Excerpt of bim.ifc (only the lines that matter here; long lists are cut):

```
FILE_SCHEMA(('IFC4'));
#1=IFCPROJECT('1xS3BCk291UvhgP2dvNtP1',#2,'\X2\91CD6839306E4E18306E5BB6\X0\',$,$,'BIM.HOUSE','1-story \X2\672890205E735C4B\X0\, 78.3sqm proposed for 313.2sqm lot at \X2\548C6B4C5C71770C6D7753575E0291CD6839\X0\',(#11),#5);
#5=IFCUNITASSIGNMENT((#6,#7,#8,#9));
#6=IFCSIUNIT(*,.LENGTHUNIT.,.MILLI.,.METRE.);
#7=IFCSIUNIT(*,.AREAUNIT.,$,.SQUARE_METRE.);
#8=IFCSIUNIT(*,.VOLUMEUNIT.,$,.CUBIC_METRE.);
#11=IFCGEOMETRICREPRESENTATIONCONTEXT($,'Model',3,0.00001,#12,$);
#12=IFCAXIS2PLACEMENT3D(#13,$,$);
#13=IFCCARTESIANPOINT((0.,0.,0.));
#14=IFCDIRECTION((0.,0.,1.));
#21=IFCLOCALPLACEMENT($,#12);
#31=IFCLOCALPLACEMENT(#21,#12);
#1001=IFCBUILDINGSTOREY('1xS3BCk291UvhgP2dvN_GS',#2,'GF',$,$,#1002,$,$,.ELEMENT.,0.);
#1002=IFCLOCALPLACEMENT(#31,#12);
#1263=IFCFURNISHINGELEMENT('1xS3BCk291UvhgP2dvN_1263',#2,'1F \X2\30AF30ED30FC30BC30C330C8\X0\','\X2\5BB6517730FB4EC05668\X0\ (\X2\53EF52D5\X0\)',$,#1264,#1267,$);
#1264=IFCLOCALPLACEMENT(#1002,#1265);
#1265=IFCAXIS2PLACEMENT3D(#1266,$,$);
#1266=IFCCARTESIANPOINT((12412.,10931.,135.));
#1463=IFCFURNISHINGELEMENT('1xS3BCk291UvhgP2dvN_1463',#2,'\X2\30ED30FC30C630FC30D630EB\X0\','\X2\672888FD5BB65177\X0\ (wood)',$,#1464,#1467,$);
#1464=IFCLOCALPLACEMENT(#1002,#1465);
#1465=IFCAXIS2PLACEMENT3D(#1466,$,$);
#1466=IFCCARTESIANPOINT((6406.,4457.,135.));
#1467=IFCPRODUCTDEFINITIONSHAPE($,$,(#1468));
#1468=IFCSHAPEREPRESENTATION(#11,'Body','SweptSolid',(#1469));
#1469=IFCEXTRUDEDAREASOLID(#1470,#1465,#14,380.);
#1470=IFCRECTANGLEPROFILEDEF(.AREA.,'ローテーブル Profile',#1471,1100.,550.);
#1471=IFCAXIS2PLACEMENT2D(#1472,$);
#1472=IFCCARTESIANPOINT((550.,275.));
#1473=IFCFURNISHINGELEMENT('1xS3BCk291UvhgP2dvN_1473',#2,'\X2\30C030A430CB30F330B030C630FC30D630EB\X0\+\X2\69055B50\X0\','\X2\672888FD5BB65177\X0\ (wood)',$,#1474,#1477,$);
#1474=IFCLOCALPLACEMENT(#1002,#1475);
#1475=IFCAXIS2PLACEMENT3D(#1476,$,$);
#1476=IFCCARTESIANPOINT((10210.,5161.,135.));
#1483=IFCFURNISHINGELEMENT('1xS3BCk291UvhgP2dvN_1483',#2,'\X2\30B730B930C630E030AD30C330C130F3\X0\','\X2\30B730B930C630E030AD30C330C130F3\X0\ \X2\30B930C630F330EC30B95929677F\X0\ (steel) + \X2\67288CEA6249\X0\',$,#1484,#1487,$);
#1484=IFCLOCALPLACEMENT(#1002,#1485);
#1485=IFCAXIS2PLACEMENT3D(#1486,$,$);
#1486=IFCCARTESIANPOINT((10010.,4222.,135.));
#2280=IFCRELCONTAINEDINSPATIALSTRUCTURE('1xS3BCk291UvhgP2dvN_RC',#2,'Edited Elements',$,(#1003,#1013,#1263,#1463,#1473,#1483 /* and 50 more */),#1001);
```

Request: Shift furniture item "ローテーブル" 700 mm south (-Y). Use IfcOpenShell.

```python
import ifcopenshell
import ifcopenshell.api.geometry
import ifcopenshell.util.placement
import ifcopenshell.util.unit

model = ifcopenshell.open("bim.ifc")
unit_scale = ifcopenshell.util.unit.calculate_unit_scale(model)

item = model.by_id(1463)
matrix = ifcopenshell.util.placement.get_local_placement(item.ObjectPlacement)
matrix[1, 3] -= 0.7 / unit_scale
ifcopenshell.api.geometry.edit_object_placement(model, product=item, matrix=matrix, is_si=False)

print(ifcopenshell.util.placement.get_local_placement(item.ObjectPlacement).round(3) + 0.0)

model.write("bim_v2.ifc")
```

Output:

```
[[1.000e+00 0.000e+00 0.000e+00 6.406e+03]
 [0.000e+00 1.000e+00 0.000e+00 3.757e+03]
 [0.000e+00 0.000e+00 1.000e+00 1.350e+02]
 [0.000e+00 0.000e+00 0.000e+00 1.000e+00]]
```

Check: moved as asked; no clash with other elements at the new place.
